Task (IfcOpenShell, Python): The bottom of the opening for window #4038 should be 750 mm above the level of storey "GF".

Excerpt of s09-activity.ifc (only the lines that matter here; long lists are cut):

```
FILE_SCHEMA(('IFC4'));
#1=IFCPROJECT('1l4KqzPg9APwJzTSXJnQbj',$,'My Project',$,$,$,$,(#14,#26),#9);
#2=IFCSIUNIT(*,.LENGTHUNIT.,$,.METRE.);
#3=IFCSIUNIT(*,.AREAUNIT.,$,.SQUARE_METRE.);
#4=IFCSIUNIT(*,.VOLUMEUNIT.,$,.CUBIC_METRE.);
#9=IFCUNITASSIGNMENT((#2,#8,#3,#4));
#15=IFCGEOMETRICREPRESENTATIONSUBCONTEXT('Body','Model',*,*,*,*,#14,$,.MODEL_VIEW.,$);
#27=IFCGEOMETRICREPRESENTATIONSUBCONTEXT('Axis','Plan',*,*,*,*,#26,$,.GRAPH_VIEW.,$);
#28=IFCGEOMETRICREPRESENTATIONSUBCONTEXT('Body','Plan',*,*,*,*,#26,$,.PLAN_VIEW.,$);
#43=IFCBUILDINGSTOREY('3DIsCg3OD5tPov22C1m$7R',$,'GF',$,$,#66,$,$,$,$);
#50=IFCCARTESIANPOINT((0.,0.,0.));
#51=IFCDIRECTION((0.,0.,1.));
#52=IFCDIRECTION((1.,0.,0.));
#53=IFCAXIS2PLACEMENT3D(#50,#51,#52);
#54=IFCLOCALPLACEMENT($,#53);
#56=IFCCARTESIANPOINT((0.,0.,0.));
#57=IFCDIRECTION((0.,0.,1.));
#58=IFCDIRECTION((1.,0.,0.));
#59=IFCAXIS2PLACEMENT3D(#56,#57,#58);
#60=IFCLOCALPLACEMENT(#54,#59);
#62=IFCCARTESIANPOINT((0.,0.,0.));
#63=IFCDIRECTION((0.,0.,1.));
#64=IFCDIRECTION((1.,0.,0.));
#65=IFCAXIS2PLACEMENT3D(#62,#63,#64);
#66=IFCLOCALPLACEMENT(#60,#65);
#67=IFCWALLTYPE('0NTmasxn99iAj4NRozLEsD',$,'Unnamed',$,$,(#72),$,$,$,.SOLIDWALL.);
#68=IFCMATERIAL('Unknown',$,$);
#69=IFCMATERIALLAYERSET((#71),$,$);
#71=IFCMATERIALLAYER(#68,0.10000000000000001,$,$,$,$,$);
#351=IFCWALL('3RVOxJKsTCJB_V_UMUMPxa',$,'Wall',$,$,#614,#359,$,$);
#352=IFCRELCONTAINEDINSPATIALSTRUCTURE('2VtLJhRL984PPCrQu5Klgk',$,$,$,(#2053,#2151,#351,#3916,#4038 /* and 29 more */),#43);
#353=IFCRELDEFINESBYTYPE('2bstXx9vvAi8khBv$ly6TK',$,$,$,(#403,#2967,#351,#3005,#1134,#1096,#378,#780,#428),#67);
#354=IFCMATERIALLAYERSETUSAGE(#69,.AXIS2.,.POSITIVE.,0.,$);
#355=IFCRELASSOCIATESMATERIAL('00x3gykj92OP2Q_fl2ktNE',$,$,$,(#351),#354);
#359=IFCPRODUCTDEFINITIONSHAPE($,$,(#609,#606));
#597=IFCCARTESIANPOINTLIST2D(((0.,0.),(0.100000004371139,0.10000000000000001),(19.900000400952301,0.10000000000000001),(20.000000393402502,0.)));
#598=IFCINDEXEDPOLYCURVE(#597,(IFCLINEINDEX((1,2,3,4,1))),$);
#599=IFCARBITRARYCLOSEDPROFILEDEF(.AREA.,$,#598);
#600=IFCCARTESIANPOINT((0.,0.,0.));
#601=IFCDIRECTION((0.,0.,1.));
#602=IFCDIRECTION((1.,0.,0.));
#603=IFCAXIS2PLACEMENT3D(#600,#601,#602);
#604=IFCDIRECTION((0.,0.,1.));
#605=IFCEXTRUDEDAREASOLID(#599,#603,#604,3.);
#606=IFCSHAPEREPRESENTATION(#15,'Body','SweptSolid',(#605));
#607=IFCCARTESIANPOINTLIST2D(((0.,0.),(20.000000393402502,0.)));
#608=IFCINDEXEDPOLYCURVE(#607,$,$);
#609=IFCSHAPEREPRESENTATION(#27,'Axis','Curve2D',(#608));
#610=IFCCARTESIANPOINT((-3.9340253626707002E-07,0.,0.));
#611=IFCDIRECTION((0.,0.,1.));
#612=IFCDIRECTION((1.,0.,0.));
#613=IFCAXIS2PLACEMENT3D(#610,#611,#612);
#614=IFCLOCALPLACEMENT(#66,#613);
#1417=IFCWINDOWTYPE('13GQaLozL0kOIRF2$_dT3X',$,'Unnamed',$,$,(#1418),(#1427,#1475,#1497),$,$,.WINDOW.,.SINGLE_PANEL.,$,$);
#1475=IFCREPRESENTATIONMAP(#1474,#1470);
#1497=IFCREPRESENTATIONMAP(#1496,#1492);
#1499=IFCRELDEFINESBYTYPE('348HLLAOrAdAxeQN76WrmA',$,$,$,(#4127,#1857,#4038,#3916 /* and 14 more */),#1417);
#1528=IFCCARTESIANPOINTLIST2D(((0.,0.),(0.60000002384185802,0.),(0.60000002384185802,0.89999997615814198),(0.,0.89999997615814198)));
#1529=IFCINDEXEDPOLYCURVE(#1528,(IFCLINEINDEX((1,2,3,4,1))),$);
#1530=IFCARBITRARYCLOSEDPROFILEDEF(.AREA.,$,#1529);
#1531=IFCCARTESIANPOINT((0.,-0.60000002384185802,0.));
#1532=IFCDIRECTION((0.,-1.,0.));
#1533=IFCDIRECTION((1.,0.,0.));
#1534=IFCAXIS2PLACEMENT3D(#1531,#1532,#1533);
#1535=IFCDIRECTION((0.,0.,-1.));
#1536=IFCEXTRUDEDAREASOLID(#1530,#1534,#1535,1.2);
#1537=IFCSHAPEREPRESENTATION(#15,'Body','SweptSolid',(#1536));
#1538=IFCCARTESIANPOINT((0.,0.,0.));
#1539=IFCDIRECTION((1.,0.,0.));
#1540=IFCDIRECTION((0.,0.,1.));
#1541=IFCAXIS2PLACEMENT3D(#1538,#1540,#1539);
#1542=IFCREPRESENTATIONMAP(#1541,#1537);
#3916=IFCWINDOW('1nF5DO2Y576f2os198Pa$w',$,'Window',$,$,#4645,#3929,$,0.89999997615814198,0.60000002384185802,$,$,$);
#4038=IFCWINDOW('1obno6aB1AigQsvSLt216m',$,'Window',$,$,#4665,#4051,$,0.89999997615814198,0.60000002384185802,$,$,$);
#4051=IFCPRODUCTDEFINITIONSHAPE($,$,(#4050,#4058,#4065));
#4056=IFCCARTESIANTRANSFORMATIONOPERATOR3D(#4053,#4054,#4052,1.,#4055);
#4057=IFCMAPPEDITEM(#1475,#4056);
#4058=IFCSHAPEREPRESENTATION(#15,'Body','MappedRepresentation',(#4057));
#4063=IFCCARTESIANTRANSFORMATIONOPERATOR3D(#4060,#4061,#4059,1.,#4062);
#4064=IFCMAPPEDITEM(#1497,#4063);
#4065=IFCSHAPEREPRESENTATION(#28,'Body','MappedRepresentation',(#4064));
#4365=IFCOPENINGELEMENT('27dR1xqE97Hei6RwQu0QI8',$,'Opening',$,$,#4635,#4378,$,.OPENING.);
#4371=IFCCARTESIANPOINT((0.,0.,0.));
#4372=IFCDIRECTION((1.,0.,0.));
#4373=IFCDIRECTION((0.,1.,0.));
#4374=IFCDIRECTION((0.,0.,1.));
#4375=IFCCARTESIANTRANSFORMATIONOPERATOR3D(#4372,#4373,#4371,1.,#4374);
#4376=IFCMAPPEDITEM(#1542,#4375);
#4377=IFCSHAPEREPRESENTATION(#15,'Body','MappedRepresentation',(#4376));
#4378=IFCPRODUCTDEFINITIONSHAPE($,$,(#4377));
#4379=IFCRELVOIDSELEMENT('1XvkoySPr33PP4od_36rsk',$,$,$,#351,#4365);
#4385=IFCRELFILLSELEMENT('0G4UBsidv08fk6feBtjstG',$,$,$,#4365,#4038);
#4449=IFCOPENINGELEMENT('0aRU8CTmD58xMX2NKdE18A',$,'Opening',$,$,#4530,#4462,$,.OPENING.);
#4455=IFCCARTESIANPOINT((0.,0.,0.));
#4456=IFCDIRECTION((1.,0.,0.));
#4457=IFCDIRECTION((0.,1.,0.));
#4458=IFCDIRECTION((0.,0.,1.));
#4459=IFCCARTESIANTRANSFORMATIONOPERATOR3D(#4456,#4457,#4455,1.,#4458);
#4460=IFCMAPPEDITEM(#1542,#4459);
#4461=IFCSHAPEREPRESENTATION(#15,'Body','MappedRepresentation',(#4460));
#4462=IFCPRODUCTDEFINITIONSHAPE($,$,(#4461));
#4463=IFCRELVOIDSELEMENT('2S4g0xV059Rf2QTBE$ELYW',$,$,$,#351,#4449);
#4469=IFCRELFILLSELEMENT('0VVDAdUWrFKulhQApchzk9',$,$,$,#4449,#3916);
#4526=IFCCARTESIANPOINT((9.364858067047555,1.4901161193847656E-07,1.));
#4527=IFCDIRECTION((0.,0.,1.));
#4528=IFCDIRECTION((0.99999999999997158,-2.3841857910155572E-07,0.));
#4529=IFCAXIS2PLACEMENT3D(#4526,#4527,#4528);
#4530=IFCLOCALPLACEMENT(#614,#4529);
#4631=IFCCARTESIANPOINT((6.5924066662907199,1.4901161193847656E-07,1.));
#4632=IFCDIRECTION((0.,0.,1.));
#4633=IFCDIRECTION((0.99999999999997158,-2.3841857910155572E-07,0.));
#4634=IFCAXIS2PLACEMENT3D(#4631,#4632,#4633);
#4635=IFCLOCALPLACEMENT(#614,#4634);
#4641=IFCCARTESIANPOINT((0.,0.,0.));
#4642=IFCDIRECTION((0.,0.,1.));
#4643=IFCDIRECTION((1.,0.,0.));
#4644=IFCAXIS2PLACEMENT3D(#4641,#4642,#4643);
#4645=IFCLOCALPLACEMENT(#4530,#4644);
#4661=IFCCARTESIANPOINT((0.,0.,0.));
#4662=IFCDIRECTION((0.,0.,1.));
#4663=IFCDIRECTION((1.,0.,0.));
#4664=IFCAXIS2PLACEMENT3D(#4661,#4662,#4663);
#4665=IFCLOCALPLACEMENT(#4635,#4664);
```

```python
import numpy as np
import ifcopenshell
import ifcopenshell.api.geometry
import ifcopenshell.geom
import ifcopenshell.util.element
import ifcopenshell.util.placement
import ifcopenshell.util.shape
import ifcopenshell.util.unit

model = ifcopenshell.open("s09-activity.ifc")
unit_scale = ifcopenshell.util.unit.calculate_unit_scale(model)

window = model.by_guid("1obno6aB1AigQsvSLt216m")
opening = window.FillsVoids[0].RelatingOpeningElement
storey = ifcopenshell.util.element.get_container(window, ifc_class="IfcBuildingStorey")
level = ifcopenshell.util.placement.get_local_placement(storey.ObjectPlacement)[2, 3]

# The opening's origin need not be at the sill, so measure its lowest point.
shape = ifcopenshell.geom.create_shape(ifcopenshell.geom.settings(), opening)
bottom = ifcopenshell.util.shape.get_shape_bottom_elevation(shape, shape.geometry) / unit_scale
dz = level + 0.75 / unit_scale - bottom

shift = np.array([0.0, 0.0, dz])
# The window is placed relative to its opening, so it follows when the opening moves.
matrix = ifcopenshell.util.placement.get_local_placement(opening.ObjectPlacement)
matrix[:3, 3] += shift
ifcopenshell.api.geometry.edit_object_placement(
    model, product=opening, matrix=matrix, is_si=False, should_transform_children=True
)

print(f"moved by {dz * unit_scale:+.3f} m")

model.write("s09-activity-out.ifc")
```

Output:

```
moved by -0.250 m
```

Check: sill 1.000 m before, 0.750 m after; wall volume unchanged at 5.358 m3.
